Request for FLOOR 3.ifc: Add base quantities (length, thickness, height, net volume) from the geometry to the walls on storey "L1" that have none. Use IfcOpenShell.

First a look at what the model holds.

```python
import ifcopenshell
import ifcopenshell.util.element
import ifcopenshell.util.unit

model = ifcopenshell.open("FLOOR 3.ifc")
print(model.schema)
for unit_type in ("LENGTHUNIT", "AREAUNIT", "VOLUMEUNIT"):
    print(unit_type, ifcopenshell.util.unit.calculate_unit_scale(model, unit_type))
storey = next(s for s in model.by_type("IfcBuildingStorey") if s.Name == "L1")
walls = [e for e in ifcopenshell.util.element.get_decomposition(storey) if e.is_a("IfcWall")]
for e in sorted(walls, key=lambda e: e.id()):
    print(e.id(), e.is_a(), e.Name, list(ifcopenshell.util.element.get_psets(e, qtos_only=True)), sep=" | ")
```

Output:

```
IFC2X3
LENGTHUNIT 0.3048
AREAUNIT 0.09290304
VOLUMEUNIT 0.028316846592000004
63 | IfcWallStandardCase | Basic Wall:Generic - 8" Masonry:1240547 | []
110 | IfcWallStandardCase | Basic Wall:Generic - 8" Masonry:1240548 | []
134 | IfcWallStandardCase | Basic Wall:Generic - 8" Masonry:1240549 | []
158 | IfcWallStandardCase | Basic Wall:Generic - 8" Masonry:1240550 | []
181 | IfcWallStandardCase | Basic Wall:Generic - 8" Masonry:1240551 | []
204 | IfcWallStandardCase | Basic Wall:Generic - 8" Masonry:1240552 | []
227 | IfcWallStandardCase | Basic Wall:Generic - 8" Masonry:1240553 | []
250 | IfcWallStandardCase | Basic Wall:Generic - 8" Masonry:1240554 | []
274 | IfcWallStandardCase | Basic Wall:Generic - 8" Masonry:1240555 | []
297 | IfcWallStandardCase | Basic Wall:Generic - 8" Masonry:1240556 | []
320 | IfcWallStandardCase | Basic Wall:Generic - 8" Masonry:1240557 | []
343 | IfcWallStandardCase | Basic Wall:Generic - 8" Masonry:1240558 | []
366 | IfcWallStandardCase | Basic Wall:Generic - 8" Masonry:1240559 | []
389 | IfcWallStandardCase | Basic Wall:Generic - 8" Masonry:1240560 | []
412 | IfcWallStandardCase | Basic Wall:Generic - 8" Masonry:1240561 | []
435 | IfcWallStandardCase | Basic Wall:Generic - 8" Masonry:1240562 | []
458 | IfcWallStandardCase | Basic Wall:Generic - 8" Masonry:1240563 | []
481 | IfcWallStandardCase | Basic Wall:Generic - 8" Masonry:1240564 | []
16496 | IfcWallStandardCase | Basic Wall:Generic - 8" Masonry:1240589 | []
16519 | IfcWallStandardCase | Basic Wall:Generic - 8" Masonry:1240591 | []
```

```python
import ifcopenshell
import ifcopenshell.api.pset
import ifcopenshell.geom
import ifcopenshell.util.element
import ifcopenshell.util.shape
import ifcopenshell.util.unit

model = ifcopenshell.open("FLOOR 3.ifc")
unit_scale = ifcopenshell.util.unit.calculate_unit_scale(model)
volume_scale = ifcopenshell.util.unit.calculate_unit_scale(model, "VOLUMEUNIT")
settings = ifcopenshell.geom.settings()

storey = next(s for s in model.by_type("IfcBuildingStorey") if s.Name == "L1")
walls = [e for e in ifcopenshell.util.element.get_decomposition(storey) if e.is_a("IfcWall")]

for e in sorted(walls, key=lambda e: e.id()):
    if ifcopenshell.util.element.get_psets(e, qtos_only=True, should_inherit=False):
        continue
    # Geometry comes back in metres, in the element's own axes.
    shape = ifcopenshell.geom.create_shape(settings, e)
    values = {
        "Length": ifcopenshell.util.shape.get_x(shape.geometry) / unit_scale,
        "Width": ifcopenshell.util.shape.get_y(shape.geometry) / unit_scale,
        "Height": ifcopenshell.util.shape.get_z(shape.geometry) / unit_scale,
        "NetVolume": ifcopenshell.util.shape.get_volume(shape.geometry) / volume_scale,
    }
    qto = ifcopenshell.api.pset.add_qto(model, product=e, name="BaseQuantities")
    ifcopenshell.api.pset.edit_qto(model, qto=qto, properties=values)
    print(e.id(), {k: round(v, 3) for k, v in values.items()})

model.write("FLOOR 3_updated.ifc")
```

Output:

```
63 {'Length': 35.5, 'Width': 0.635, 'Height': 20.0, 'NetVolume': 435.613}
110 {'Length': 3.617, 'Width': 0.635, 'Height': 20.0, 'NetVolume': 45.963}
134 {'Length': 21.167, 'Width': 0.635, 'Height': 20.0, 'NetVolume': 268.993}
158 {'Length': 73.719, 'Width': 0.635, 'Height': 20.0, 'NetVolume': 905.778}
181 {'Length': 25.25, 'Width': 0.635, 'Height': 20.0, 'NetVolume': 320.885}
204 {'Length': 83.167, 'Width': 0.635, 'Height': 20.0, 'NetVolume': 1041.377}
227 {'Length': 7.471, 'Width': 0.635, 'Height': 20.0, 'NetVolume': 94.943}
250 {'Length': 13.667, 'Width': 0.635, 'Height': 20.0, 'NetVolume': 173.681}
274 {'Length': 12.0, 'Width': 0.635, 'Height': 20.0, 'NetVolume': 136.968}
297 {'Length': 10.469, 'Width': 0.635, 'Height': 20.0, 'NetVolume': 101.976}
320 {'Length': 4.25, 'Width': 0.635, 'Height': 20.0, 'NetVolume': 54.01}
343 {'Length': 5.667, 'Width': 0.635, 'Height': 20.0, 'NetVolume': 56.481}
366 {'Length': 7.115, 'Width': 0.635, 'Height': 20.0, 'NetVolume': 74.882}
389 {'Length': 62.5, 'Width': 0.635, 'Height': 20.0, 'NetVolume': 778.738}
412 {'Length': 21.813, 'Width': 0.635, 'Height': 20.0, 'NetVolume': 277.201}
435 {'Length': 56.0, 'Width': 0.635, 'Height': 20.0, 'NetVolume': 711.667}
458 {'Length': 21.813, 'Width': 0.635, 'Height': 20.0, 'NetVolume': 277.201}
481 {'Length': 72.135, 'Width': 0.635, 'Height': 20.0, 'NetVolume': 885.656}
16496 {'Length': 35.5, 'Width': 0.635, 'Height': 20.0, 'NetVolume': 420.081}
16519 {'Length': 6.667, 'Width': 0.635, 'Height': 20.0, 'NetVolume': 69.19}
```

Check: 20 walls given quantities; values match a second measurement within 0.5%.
